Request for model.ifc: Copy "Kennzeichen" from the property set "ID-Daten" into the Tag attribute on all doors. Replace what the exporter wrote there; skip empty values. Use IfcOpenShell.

First a look at what the model holds.

```python
import ifcopenshell
import ifcopenshell.util.element

model = ifcopenshell.open("model.ifc")
print(model.schema)
doors = model.by_type("IfcDoor")
print(len(doors), "doors")
for e in doors[:8]:
    source = ifcopenshell.util.element.get_pset(e, "ID-Daten", "Kennzeichen")
    target = e.Tag
    print(e.id(), repr(source), repr(target), sep=" | ")
```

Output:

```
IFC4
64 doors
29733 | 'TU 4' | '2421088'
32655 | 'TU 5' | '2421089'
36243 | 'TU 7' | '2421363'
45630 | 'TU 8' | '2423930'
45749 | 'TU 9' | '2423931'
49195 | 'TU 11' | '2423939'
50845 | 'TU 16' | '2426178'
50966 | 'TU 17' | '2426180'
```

```python
import ifcopenshell
import ifcopenshell.util.element

model = ifcopenshell.open("model.ifc")

count = 0
for e in model.by_type("IfcDoor"):
    value = ifcopenshell.util.element.get_pset(e, "ID-Daten", "Kennzeichen")
    current = e.Tag
    if not value or not value.strip() or current == value:
        continue
    e.Tag = value
    count += 1

print(count, "doors updated")

model.write("model_rev.ifc")
```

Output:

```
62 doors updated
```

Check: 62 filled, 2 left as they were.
